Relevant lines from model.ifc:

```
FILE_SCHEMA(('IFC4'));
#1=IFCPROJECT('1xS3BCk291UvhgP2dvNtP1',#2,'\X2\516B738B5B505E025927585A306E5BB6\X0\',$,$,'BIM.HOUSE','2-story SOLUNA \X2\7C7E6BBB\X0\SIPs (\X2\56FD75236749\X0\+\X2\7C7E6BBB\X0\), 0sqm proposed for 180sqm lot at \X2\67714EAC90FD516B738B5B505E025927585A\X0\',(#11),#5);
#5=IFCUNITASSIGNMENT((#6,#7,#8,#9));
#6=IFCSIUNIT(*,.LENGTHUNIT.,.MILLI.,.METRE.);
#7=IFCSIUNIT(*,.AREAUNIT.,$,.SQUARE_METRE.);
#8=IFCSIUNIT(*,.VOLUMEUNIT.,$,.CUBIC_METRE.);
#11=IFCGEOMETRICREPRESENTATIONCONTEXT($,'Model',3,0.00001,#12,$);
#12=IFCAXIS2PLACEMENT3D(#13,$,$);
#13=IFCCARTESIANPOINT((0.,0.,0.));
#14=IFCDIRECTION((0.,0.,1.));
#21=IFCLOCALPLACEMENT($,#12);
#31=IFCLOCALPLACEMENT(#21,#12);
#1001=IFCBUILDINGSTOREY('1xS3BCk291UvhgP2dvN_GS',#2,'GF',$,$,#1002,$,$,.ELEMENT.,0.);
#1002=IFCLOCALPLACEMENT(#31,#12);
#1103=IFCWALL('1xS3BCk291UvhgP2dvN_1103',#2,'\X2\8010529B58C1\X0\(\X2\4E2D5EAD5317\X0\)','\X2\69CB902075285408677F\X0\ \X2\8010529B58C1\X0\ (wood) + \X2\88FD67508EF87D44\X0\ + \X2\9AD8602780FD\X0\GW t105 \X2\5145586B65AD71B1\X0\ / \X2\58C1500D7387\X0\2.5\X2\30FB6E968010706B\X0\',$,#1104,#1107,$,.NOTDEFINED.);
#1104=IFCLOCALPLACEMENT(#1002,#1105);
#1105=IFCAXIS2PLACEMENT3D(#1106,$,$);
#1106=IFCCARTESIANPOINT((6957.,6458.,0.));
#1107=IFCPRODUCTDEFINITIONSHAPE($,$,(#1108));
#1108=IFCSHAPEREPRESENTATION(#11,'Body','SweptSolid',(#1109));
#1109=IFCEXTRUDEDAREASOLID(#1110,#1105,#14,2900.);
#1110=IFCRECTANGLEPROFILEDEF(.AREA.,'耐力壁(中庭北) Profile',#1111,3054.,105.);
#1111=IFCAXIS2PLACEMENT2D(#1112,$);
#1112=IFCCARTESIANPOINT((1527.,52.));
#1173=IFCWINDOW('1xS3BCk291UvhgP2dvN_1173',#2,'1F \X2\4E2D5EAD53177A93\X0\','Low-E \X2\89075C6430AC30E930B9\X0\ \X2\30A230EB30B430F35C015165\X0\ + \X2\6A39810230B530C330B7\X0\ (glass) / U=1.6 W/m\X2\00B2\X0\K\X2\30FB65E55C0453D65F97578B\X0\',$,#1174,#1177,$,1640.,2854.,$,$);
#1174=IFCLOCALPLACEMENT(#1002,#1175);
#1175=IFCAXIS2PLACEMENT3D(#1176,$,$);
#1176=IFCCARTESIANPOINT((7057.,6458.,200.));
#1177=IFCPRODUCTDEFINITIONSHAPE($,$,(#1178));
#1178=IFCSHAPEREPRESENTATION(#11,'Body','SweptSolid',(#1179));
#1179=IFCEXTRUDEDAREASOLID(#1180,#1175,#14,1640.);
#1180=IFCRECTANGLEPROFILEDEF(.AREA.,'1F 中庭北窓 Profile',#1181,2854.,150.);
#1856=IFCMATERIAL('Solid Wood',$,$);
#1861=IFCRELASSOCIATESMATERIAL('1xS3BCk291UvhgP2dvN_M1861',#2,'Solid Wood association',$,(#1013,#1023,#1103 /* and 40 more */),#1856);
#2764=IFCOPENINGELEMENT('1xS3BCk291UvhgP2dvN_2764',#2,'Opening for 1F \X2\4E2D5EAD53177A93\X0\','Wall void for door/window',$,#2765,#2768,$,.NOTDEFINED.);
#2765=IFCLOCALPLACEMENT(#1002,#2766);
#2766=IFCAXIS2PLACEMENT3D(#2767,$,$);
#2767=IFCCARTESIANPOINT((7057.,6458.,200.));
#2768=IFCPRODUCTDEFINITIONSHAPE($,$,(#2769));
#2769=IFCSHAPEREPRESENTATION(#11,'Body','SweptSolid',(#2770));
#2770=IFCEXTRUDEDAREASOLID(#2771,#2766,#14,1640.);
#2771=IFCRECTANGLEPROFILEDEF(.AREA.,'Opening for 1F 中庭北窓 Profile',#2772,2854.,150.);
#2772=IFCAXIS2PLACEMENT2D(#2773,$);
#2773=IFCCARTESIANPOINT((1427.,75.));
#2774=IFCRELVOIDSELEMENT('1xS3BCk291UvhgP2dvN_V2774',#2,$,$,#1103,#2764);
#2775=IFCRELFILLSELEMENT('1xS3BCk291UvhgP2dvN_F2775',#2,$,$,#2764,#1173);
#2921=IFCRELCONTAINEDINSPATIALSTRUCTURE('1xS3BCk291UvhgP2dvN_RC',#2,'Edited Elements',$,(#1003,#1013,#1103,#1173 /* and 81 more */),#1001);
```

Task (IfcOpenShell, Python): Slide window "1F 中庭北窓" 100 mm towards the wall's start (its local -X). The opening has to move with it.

```python
import ifcopenshell
import ifcopenshell.api.geometry
import ifcopenshell.util.placement
import ifcopenshell.util.unit

model = ifcopenshell.open("model.ifc")
unit_scale = ifcopenshell.util.unit.calculate_unit_scale(model)

window = model.by_guid("1xS3BCk291UvhgP2dvN_1173")
opening = window.FillsVoids[0].RelatingOpeningElement
wall = opening.VoidsElements[0].RelatingBuildingElement

wall_matrix = ifcopenshell.util.placement.get_local_placement(wall.ObjectPlacement)
shift = wall_matrix[:3, 0] * -0.1 / unit_scale
before = ifcopenshell.util.placement.get_local_placement(window.ObjectPlacement)[:3, 3].copy()

# The window is not placed relative to its opening, so move both.
for product in (opening, window):
    matrix = ifcopenshell.util.placement.get_local_placement(product.ObjectPlacement)
    matrix[:3, 3] += shift
    ifcopenshell.api.geometry.edit_object_placement(model, product=product, matrix=matrix, is_si=False)

after = ifcopenshell.util.placement.get_local_placement(window.ObjectPlacement)[:3, 3]
print("window moved by", (after - before).round(3) + 0.0)

model.write("model_updated.ifc")
```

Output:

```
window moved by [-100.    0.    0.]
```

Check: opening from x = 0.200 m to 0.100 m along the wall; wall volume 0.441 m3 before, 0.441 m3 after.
